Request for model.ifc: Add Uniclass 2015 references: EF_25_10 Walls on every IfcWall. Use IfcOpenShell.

First a look at what the model holds.

```python
import ifcopenshell

model = ifcopenshell.open("model.ifc")
print(model.schema)
print("classifications:", [c.Name for c in model.by_type("IfcClassification")])
for ifc_class in ("IfcDoor", "IfcRoof", "IfcStair", "IfcWall", "IfcWindow"):
    print(ifc_class, len(model.by_type(ifc_class)))
```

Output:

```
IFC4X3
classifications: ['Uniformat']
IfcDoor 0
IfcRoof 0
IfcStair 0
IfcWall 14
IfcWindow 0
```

```python
import ifcopenshell
import ifcopenshell.api.classification

model = ifcopenshell.open("model.ifc")

system = ifcopenshell.api.classification.add_classification(model, classification="Uniclass 2015")

codes = {
    "IfcWall": ("EF_25_10", "Walls"),
}
for ifc_class, (code, name) in codes.items():
    products = model.by_type(ifc_class)
    ifcopenshell.api.classification.add_reference(
        model, products=products, classification=system, identification=code, name=name
    )
    print(code, len(products))

model.write("model_edited.ifc")
```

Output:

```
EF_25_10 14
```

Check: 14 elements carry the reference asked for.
